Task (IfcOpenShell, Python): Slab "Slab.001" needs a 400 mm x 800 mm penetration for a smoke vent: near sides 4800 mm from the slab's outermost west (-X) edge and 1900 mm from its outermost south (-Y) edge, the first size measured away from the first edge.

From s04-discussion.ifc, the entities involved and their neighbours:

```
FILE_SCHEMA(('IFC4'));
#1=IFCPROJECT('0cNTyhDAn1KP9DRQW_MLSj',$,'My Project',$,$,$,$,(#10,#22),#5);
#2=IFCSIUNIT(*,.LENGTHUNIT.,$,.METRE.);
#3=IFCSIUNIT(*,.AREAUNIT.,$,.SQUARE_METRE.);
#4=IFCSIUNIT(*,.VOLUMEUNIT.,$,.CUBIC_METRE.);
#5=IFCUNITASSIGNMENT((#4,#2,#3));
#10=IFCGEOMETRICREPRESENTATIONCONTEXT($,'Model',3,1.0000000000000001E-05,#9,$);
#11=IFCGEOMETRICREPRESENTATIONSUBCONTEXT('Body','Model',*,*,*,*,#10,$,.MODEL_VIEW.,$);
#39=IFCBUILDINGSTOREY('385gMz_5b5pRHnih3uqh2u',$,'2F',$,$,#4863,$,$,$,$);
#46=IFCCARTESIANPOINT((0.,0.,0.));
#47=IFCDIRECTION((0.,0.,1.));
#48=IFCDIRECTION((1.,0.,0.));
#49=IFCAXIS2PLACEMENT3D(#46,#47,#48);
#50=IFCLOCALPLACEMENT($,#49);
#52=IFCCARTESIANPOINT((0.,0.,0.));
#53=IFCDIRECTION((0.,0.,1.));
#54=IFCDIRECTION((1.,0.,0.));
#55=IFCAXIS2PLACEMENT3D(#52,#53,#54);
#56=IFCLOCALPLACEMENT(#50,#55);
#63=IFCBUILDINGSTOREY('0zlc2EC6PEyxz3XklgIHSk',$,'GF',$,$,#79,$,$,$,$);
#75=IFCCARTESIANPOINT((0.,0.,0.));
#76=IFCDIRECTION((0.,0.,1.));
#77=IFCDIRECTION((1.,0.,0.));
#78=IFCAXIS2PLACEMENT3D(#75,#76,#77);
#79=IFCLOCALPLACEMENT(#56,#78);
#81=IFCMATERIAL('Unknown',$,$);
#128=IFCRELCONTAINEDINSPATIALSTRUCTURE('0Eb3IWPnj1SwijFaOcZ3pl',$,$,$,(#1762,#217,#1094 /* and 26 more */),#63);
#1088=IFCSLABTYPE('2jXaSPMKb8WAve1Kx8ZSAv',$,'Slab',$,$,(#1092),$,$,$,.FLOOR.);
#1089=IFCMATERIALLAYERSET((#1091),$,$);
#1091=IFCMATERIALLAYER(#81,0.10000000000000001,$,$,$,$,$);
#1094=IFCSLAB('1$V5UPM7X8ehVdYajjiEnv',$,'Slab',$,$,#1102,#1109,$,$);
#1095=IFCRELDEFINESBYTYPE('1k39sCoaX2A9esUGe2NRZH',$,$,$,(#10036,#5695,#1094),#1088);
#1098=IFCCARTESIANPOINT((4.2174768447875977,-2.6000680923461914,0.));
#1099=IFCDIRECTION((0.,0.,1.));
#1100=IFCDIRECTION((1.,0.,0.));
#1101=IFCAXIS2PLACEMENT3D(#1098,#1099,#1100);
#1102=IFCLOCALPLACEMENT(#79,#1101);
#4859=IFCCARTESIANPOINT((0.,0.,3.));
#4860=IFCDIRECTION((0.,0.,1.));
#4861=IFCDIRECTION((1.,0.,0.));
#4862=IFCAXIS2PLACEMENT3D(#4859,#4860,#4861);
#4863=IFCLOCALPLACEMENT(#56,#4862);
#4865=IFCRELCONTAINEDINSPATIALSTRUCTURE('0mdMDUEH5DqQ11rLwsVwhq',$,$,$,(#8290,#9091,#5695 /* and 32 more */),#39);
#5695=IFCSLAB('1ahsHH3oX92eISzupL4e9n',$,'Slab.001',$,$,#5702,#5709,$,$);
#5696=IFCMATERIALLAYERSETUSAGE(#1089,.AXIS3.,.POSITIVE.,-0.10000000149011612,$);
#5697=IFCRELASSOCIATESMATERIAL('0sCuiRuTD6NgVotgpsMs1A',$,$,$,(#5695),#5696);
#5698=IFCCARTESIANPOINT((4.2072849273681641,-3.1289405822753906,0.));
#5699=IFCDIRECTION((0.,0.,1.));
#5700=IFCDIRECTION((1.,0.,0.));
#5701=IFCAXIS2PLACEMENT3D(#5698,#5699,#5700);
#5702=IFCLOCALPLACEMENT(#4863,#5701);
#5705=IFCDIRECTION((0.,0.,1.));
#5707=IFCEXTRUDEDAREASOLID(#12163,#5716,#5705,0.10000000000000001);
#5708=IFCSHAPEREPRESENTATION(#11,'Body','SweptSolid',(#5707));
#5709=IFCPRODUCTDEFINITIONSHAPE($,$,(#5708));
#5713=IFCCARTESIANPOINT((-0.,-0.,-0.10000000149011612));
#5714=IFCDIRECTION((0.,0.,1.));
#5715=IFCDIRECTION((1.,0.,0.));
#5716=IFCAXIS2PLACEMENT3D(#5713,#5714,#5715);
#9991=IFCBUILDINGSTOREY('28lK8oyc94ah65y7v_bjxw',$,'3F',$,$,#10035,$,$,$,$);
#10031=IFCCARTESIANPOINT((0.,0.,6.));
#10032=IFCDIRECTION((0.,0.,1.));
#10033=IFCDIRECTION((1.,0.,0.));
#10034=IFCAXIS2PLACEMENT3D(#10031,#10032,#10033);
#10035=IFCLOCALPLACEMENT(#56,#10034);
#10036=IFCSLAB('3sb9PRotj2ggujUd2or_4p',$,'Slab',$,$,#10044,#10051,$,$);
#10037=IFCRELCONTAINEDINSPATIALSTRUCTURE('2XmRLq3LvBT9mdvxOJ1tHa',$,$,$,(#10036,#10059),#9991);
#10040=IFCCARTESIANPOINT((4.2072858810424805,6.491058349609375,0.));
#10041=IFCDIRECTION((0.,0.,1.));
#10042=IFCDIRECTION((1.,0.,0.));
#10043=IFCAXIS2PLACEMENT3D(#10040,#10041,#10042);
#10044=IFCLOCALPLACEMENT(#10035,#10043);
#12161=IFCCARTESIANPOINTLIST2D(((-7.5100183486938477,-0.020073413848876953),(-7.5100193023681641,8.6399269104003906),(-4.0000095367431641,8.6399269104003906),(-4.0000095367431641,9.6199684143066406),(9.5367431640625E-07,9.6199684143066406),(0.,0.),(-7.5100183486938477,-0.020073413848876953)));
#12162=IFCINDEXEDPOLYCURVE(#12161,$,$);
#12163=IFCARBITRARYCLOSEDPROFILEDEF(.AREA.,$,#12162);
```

```python
import numpy as np
import ifcopenshell
import ifcopenshell.api.feature
import ifcopenshell.api.geometry
import ifcopenshell.api.root
import ifcopenshell.geom
import ifcopenshell.util.placement
import ifcopenshell.util.representation
import ifcopenshell.util.shape
import ifcopenshell.util.unit

model = ifcopenshell.open("s04-discussion.ifc")
unit_scale = ifcopenshell.util.unit.calculate_unit_scale(model)
settings = ifcopenshell.geom.settings()


def volume(element):
    """Net volume in cubic metres, openings subtracted."""
    shape = ifcopenshell.geom.create_shape(settings, element)
    return ifcopenshell.util.shape.get_volume(shape.geometry)


slab = model.by_guid("1ahsHH3oX92eISzupL4e9n")
before = volume(slab)

# Extent in the slab's own axes, in metres. The edges named are its -X and -Y sides.
slab_shape = ifcopenshell.geom.create_shape(settings, slab)
vertices = ifcopenshell.util.shape.get_vertices(slab_shape.geometry)
x_min, y_min, bottom = vertices.min(axis=0)
top = vertices[:, 2].max()

opening = ifcopenshell.api.root.create_entity(model, ifc_class="IfcOpeningElement", name="Smoke vent opening", predefined_type="OPENING")
context = ifcopenshell.util.representation.get_context(model, "Model", "Body", "MODEL_VIEW")
width, depth = 0.4, 0.8
outline = [(0.0, 0.0), (width, 0.0), (width, depth), (0.0, depth), (0.0, 0.0)]
# Overshoot both faces by 50 mm so the cut is clean.
shape = ifcopenshell.api.geometry.add_slab_representation(
    model, context=context, depth=top - bottom + 0.1, polyline=outline
)
ifcopenshell.api.geometry.assign_representation(model, product=opening, representation=shape)

matrix = ifcopenshell.util.placement.get_local_placement(slab.ObjectPlacement)
matrix[:, 3] = matrix @ np.append(np.array([x_min + 4.8, y_min + 1.9, bottom - 0.05]) / unit_scale, 1.0)
ifcopenshell.api.geometry.edit_object_placement(model, product=opening, matrix=matrix, is_si=False)
ifcopenshell.api.feature.add_feature(model, feature=opening, element=slab)

after = volume(slab)

print(f"slab volume {before:.3f} -> {after:.3f} m3")

model.write("s04-discussion_rev.ifc")
```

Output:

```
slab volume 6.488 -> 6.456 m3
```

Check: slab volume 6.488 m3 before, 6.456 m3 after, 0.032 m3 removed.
